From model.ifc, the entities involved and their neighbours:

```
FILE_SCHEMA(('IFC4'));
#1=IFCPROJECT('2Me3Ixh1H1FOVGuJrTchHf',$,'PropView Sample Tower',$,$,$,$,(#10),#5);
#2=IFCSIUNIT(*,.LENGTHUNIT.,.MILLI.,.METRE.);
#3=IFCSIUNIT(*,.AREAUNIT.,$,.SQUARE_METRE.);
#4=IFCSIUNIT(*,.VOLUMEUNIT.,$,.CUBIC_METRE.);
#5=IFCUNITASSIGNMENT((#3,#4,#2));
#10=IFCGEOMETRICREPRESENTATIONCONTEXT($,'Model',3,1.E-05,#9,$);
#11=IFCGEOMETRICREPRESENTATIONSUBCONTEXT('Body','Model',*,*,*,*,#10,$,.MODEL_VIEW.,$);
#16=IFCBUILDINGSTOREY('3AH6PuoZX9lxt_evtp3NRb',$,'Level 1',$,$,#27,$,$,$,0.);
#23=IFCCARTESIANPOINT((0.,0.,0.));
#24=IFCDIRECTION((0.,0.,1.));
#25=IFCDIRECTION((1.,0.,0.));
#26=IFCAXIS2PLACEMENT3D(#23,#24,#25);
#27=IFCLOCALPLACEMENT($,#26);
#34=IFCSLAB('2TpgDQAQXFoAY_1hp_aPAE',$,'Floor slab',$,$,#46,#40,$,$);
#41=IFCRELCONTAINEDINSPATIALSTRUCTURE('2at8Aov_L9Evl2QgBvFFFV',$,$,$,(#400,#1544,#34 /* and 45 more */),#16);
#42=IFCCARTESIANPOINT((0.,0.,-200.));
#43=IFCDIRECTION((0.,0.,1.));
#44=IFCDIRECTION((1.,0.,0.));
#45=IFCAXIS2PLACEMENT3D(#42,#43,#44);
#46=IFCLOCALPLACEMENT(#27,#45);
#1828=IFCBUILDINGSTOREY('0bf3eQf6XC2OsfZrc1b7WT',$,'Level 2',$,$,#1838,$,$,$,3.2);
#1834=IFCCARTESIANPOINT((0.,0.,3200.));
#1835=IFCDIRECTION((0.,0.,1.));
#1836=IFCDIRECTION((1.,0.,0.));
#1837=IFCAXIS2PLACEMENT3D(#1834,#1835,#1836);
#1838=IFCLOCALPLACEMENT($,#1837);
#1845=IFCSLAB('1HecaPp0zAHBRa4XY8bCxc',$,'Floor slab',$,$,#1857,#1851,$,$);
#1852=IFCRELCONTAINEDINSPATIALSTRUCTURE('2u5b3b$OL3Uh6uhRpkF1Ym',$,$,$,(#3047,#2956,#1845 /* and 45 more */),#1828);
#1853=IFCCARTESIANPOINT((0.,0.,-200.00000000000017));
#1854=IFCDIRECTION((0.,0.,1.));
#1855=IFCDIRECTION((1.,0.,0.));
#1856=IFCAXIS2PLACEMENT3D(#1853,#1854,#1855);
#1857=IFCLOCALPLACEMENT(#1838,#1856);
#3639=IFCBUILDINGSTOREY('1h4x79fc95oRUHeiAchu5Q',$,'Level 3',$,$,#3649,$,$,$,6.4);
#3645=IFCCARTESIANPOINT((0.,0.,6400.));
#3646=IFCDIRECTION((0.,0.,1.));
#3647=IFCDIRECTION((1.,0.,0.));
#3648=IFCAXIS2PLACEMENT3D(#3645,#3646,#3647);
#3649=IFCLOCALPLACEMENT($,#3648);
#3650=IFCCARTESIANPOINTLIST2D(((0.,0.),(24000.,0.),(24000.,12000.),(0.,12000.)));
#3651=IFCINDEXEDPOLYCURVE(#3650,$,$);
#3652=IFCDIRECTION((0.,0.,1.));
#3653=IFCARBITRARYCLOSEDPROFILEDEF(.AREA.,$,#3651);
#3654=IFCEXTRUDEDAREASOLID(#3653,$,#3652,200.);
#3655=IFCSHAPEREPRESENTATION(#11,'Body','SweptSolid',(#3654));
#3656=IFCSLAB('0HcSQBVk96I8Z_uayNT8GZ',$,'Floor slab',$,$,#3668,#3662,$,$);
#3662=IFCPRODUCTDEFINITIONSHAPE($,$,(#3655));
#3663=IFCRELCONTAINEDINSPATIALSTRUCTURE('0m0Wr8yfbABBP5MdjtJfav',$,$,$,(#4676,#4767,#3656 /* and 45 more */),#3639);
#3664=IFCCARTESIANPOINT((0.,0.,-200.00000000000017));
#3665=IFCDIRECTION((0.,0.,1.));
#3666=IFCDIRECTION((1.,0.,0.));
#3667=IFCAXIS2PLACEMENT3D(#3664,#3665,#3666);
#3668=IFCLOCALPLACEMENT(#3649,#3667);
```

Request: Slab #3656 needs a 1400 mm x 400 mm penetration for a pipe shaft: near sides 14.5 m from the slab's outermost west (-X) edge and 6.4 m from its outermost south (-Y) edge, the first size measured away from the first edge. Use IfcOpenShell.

```python
import numpy as np
import ifcopenshell
import ifcopenshell.api.feature
import ifcopenshell.api.geometry
import ifcopenshell.api.root
import ifcopenshell.geom
import ifcopenshell.util.placement
import ifcopenshell.util.representation
import ifcopenshell.util.shape
import ifcopenshell.util.unit

model = ifcopenshell.open("model.ifc")
unit_scale = ifcopenshell.util.unit.calculate_unit_scale(model)
settings = ifcopenshell.geom.settings()


def volume(element):
    """Net volume in cubic metres, openings subtracted."""
    shape = ifcopenshell.geom.create_shape(settings, element)
    return ifcopenshell.util.shape.get_volume(shape.geometry)


slab = model.by_id(3656)
before = volume(slab)

# Extent in the slab's own axes, in metres. The edges named are its -X and -Y sides.
slab_shape = ifcopenshell.geom.create_shape(settings, slab)
vertices = ifcopenshell.util.shape.get_vertices(slab_shape.geometry)
x_min, y_min, bottom = vertices.min(axis=0)
top = vertices[:, 2].max()

opening = ifcopenshell.api.root.create_entity(model, ifc_class="IfcOpeningElement", name="Pipe shaft opening", predefined_type="OPENING")
context = ifcopenshell.util.representation.get_context(model, "Model", "Body", "MODEL_VIEW")
width, depth = 1.4, 0.4
outline = [(0.0, 0.0), (width, 0.0), (width, depth), (0.0, depth), (0.0, 0.0)]
# Overshoot both faces by 50 mm so the cut is clean.
shape = ifcopenshell.api.geometry.add_slab_representation(
    model, context=context, depth=top - bottom + 0.1, polyline=outline
)
ifcopenshell.api.geometry.assign_representation(model, product=opening, representation=shape)

matrix = ifcopenshell.util.placement.get_local_placement(slab.ObjectPlacement)
matrix[:, 3] = matrix @ np.append(np.array([x_min + 14.5, y_min + 6.4, bottom - 0.05]) / unit_scale, 1.0)
ifcopenshell.api.geometry.edit_object_placement(model, product=opening, matrix=matrix, is_si=False)
ifcopenshell.api.feature.add_feature(model, feature=opening, element=slab)

after = volume(slab)

print(f"slab volume {before:.3f} -> {after:.3f} m3")

model.write("model_rev.ifc")
```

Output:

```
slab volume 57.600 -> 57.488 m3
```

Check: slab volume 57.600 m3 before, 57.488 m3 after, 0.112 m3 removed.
